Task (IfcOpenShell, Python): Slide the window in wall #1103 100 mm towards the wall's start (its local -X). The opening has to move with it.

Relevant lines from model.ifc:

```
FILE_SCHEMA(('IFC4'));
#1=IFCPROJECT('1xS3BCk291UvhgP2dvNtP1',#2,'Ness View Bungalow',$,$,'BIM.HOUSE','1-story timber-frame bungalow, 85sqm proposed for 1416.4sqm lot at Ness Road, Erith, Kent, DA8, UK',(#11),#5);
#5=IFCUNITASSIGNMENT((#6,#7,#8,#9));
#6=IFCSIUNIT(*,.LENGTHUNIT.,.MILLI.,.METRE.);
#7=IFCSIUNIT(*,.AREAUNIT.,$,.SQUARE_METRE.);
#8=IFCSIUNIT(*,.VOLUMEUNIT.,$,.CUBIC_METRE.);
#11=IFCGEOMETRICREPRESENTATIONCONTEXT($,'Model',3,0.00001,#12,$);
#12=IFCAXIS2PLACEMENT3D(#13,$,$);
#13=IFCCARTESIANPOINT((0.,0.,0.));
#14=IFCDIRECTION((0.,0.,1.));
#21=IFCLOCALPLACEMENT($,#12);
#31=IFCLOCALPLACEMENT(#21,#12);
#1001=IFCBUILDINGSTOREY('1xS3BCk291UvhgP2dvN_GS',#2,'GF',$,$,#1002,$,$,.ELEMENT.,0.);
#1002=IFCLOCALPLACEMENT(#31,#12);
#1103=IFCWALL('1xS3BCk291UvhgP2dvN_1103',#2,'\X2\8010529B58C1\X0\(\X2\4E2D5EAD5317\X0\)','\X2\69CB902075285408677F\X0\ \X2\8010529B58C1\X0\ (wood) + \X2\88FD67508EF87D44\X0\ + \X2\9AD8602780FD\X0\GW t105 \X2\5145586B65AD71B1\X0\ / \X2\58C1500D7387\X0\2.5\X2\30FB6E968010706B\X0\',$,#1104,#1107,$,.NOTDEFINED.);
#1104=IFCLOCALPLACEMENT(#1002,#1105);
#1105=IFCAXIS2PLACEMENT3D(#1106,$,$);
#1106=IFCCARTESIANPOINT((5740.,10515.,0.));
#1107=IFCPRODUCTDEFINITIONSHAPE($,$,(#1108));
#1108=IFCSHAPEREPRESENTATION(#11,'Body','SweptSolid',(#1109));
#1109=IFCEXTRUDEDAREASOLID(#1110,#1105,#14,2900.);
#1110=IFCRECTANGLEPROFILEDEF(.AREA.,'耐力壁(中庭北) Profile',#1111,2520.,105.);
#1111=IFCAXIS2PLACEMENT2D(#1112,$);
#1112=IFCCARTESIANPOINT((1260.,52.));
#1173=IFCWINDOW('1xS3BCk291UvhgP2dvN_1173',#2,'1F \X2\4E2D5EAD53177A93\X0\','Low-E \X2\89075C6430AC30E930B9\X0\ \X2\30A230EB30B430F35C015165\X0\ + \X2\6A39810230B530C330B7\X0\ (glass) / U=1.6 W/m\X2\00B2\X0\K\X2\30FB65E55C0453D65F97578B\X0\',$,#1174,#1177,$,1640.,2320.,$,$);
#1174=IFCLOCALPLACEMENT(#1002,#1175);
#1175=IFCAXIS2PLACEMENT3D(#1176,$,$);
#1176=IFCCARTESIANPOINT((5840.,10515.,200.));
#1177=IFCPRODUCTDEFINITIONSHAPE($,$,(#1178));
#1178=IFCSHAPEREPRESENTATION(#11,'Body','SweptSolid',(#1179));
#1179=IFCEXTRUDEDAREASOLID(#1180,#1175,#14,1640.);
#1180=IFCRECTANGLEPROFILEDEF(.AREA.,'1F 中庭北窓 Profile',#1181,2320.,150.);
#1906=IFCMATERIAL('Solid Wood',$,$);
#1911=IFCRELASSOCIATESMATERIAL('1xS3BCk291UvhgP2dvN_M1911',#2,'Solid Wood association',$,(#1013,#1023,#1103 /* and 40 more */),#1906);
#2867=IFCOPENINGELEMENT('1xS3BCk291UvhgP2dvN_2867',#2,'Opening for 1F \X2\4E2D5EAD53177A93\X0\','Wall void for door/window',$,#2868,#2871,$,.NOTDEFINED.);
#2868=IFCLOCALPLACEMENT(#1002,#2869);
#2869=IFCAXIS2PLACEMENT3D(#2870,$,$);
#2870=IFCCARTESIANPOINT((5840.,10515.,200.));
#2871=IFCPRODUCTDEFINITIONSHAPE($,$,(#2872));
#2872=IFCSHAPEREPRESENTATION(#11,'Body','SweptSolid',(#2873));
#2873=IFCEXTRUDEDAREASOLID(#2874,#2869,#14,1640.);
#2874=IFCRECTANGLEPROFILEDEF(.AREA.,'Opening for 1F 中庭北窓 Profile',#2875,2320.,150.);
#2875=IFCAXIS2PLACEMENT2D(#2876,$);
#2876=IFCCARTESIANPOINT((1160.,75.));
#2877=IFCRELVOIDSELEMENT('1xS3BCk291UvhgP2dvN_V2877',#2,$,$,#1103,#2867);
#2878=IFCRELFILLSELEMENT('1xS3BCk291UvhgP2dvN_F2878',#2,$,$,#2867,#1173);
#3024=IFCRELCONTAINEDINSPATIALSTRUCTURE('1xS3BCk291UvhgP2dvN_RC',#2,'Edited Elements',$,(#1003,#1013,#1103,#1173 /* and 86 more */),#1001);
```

```python
import ifcopenshell
import ifcopenshell.api.geometry
import ifcopenshell.util.placement

model = ifcopenshell.open("model.ifc")

window = model.by_id(1173)
opening = window.FillsVoids[0].RelatingOpeningElement
wall = opening.VoidsElements[0].RelatingBuildingElement

wall_matrix = ifcopenshell.util.placement.get_local_placement(wall.ObjectPlacement)
shift = wall_matrix[:3, 0] * -100.0
before = ifcopenshell.util.placement.get_local_placement(window.ObjectPlacement)[:3, 3].copy()

# The window is not placed relative to its opening, so move both.
for product in (opening, window):
    matrix = ifcopenshell.util.placement.get_local_placement(product.ObjectPlacement)
    matrix[:3, 3] += shift
    ifcopenshell.api.geometry.edit_object_placement(model, product=product, matrix=matrix, is_si=False)

after = ifcopenshell.util.placement.get_local_placement(window.ObjectPlacement)[:3, 3]
print("window moved by", (after - before).round(3) + 0.0)

model.write("model_rev.ifc")
```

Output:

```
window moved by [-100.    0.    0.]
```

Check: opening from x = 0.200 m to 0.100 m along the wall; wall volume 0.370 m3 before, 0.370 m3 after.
